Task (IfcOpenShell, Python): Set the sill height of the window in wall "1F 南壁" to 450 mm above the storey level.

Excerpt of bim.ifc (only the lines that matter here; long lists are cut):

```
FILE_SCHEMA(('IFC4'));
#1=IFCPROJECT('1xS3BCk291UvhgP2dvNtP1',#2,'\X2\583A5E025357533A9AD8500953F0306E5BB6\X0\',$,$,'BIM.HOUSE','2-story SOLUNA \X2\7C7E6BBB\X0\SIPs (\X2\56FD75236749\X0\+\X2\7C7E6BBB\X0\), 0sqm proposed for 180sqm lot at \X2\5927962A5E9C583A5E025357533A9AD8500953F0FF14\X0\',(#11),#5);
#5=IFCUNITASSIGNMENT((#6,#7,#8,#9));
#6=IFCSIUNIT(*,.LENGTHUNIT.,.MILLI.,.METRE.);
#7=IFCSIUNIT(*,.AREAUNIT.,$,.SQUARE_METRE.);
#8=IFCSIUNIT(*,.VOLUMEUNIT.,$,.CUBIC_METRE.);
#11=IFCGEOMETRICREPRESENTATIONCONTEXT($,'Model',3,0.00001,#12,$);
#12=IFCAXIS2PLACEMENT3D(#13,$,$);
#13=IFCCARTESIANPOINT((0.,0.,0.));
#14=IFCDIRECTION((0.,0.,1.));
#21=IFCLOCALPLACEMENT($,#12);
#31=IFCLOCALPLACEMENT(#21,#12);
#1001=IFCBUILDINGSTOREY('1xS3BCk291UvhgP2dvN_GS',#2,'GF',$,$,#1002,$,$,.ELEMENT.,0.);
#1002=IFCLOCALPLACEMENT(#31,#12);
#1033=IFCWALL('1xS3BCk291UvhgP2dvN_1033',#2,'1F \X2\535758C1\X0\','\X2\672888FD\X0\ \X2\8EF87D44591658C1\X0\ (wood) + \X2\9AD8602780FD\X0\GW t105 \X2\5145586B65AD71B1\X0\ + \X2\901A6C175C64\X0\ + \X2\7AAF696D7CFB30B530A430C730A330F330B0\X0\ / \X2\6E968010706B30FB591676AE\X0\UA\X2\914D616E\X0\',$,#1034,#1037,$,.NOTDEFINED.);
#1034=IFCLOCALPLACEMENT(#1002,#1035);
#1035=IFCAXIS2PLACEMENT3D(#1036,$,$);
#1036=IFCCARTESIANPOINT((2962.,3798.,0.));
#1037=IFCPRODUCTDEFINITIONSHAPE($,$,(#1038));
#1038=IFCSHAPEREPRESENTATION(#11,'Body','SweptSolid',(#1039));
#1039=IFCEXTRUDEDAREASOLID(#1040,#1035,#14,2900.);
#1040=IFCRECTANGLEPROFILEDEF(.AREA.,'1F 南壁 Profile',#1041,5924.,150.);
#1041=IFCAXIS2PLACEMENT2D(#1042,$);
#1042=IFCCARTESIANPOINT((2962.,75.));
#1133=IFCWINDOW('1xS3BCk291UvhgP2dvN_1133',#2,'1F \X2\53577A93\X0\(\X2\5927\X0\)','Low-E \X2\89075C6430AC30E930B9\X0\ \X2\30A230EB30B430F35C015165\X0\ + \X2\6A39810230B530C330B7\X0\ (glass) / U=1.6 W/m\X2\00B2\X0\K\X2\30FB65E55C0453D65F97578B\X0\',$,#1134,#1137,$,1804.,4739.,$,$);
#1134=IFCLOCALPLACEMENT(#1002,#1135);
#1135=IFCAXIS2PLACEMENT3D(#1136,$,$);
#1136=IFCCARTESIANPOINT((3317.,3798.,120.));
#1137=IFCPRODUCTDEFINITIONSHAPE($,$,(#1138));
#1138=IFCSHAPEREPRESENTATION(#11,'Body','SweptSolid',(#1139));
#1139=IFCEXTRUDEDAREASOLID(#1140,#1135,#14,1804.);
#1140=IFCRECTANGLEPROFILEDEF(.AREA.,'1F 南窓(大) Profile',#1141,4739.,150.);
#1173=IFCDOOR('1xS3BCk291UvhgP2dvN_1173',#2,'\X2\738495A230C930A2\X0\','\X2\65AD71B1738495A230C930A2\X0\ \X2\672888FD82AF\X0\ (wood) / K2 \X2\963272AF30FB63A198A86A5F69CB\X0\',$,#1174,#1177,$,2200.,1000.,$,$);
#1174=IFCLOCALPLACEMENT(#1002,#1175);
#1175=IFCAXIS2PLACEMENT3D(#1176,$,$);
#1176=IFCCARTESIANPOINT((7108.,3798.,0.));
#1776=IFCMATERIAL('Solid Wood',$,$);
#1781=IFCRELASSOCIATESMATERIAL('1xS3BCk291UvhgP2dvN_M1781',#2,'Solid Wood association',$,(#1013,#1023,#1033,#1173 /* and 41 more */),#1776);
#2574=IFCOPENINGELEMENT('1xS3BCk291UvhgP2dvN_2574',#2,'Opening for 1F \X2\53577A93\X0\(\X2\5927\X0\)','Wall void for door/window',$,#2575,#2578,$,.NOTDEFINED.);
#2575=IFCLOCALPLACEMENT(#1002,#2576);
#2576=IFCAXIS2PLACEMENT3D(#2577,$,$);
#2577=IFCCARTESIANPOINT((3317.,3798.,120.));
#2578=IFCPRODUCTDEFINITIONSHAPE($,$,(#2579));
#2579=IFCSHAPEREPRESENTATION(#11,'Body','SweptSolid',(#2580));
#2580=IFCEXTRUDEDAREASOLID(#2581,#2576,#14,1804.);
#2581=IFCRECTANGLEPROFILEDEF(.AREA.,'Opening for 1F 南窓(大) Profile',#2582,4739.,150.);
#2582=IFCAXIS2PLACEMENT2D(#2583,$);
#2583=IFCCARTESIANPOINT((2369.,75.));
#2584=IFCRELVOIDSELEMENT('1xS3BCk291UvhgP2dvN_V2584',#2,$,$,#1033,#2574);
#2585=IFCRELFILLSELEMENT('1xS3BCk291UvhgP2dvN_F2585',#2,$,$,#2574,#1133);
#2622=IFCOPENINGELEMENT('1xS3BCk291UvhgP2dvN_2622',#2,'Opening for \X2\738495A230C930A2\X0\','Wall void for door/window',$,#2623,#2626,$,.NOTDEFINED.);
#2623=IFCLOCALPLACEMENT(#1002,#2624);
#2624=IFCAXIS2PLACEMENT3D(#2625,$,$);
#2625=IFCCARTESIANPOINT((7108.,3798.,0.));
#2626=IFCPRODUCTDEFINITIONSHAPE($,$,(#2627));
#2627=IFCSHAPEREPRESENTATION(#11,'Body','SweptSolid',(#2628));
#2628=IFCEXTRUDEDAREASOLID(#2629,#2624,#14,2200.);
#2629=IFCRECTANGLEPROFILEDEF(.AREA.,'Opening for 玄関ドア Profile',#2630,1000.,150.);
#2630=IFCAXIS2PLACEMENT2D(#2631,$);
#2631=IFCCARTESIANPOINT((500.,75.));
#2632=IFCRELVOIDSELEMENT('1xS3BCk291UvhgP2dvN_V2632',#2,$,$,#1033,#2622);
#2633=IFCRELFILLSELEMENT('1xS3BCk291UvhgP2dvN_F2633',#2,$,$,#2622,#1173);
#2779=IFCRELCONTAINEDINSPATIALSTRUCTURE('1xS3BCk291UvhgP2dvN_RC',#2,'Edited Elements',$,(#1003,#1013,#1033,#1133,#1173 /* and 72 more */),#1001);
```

```python
import numpy as np
import ifcopenshell
import ifcopenshell.api.geometry
import ifcopenshell.geom
import ifcopenshell.util.element
import ifcopenshell.util.placement
import ifcopenshell.util.shape
import ifcopenshell.util.unit

model = ifcopenshell.open("bim.ifc")
unit_scale = ifcopenshell.util.unit.calculate_unit_scale(model)

window = model.by_guid("1xS3BCk291UvhgP2dvN_1133")
opening = window.FillsVoids[0].RelatingOpeningElement
storey = ifcopenshell.util.element.get_container(window, ifc_class="IfcBuildingStorey")
level = ifcopenshell.util.placement.get_local_placement(storey.ObjectPlacement)[2, 3]

# The opening's origin need not be at the sill, so measure its lowest point.
shape = ifcopenshell.geom.create_shape(ifcopenshell.geom.settings(), opening)
bottom = ifcopenshell.util.shape.get_shape_bottom_elevation(shape, shape.geometry) / unit_scale
dz = level + 450.0 - bottom

shift = np.array([0.0, 0.0, dz])
# The window is not placed relative to its opening, so move both.
for product in (opening, window):
    matrix = ifcopenshell.util.placement.get_local_placement(product.ObjectPlacement)
    matrix[:3, 3] += shift
    ifcopenshell.api.geometry.edit_object_placement(model, product=product, matrix=matrix, is_si=False)

print(f"moved by {dz * unit_scale:+.3f} m")

model.write("bim-out.ifc")
```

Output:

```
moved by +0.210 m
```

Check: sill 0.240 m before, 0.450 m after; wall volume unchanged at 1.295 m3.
